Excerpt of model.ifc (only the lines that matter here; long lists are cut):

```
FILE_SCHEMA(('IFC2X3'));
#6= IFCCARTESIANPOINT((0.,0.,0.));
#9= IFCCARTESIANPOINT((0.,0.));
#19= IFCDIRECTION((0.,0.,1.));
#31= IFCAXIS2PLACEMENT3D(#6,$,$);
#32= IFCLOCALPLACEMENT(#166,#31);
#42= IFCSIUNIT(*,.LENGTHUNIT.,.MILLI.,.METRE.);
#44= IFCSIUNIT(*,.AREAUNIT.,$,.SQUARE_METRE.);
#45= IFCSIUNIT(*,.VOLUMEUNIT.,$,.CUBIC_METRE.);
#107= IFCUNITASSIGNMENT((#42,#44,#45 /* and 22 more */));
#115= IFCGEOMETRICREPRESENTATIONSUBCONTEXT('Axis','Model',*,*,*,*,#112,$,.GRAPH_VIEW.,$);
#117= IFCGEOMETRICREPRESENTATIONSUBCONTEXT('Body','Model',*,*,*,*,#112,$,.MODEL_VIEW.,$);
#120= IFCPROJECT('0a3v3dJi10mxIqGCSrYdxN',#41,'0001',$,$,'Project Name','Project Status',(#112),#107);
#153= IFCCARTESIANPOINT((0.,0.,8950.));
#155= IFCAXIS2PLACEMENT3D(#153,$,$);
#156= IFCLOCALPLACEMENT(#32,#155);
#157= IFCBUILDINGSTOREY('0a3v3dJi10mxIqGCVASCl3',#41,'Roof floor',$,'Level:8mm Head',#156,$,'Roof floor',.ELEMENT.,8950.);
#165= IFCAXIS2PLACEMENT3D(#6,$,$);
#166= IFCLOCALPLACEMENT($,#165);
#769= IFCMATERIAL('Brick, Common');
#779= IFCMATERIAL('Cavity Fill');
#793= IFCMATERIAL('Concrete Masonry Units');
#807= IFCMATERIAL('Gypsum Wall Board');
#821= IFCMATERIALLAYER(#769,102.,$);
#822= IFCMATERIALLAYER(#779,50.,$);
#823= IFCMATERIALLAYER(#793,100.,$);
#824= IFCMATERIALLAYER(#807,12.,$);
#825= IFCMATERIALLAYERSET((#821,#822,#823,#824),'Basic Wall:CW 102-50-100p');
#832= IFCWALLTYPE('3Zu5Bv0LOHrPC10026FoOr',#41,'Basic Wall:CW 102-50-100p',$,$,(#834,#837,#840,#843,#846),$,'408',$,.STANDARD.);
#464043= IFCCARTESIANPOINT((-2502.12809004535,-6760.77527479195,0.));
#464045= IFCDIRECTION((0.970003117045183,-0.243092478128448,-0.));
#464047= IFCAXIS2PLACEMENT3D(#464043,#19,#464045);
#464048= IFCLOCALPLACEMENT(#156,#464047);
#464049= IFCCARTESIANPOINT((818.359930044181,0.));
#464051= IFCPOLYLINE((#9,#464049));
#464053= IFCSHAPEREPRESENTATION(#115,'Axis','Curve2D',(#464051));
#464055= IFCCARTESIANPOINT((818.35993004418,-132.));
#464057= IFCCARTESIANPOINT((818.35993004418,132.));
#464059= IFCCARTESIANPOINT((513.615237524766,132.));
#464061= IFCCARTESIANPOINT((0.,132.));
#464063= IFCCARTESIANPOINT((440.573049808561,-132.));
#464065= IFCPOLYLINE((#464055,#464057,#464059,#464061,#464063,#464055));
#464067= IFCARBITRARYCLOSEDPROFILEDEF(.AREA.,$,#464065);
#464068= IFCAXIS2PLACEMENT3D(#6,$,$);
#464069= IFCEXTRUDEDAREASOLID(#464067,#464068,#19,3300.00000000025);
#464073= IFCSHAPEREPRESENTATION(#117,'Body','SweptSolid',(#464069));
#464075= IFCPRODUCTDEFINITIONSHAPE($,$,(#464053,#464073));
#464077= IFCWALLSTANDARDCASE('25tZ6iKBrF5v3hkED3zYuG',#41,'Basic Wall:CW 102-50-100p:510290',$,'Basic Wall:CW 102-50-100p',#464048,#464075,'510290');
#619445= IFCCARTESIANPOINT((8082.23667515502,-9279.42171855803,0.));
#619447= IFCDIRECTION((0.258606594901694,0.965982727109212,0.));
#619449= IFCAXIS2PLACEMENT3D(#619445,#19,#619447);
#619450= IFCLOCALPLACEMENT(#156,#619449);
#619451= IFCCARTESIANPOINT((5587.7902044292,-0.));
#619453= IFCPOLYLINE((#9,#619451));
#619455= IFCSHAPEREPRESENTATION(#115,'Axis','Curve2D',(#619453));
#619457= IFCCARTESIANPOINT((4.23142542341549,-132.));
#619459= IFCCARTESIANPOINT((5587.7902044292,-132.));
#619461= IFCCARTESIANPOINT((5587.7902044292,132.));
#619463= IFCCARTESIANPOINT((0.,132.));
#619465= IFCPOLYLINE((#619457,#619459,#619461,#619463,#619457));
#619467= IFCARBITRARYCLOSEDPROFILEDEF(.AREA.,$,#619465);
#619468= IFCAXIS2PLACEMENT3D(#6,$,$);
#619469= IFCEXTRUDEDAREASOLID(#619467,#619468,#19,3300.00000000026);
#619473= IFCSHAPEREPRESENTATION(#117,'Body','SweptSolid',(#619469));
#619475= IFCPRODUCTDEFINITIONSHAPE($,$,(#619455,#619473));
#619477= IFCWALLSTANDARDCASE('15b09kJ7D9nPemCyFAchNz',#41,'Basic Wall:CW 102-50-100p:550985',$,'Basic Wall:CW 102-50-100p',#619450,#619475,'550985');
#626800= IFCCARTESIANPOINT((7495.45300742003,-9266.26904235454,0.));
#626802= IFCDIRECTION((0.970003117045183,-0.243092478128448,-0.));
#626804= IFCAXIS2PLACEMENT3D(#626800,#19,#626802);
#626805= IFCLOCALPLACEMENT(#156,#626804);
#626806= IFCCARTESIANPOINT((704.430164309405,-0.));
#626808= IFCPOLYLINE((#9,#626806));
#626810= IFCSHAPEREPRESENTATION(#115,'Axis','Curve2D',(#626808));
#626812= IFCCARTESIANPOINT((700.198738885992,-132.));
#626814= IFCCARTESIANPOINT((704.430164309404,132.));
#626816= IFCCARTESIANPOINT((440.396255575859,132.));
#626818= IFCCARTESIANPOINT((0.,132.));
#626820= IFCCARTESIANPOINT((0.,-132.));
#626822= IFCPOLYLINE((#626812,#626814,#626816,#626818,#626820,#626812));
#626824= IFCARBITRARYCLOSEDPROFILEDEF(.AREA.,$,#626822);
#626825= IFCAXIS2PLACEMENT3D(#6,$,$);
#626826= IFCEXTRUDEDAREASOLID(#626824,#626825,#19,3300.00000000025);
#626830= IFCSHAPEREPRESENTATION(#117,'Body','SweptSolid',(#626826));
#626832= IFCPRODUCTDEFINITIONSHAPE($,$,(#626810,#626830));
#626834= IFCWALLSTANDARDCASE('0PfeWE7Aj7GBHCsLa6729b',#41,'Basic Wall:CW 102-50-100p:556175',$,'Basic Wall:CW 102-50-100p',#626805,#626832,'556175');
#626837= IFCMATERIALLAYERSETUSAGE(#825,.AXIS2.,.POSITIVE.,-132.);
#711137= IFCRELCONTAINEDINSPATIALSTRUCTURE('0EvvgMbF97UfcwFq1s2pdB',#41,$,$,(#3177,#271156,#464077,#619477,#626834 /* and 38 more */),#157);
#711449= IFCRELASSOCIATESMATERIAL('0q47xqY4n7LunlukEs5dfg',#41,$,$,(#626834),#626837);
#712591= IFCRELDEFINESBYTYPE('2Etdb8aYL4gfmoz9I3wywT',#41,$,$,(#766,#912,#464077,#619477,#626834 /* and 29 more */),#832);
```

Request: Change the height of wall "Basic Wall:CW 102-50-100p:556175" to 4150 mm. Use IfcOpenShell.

```python
import ifcopenshell
import ifcopenshell.geom
import ifcopenshell.util.representation
import ifcopenshell.util.shape

model = ifcopenshell.open("model.ifc")
settings = ifcopenshell.geom.settings()


def volume(element):
    """Net volume in cubic metres, openings subtracted."""
    shape = ifcopenshell.geom.create_shape(settings, element)
    return ifcopenshell.util.shape.get_volume(shape.geometry)


wall = model.by_guid("0PfeWE7Aj7GBHCsLa6729b")
before = volume(wall)

body = ifcopenshell.util.representation.get_representation(wall, "Model", "Body")
solid = body.Items[0]
old_height = solid.Depth
solid.Depth = 4150.0
after = volume(wall)

print(f"height {old_height:g} -> {solid.Depth:g}, volume {before:.3f} -> {after:.3f} m3")

model.write("model_v2.ifc")
```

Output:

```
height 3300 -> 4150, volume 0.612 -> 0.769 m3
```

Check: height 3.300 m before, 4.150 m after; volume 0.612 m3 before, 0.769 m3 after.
